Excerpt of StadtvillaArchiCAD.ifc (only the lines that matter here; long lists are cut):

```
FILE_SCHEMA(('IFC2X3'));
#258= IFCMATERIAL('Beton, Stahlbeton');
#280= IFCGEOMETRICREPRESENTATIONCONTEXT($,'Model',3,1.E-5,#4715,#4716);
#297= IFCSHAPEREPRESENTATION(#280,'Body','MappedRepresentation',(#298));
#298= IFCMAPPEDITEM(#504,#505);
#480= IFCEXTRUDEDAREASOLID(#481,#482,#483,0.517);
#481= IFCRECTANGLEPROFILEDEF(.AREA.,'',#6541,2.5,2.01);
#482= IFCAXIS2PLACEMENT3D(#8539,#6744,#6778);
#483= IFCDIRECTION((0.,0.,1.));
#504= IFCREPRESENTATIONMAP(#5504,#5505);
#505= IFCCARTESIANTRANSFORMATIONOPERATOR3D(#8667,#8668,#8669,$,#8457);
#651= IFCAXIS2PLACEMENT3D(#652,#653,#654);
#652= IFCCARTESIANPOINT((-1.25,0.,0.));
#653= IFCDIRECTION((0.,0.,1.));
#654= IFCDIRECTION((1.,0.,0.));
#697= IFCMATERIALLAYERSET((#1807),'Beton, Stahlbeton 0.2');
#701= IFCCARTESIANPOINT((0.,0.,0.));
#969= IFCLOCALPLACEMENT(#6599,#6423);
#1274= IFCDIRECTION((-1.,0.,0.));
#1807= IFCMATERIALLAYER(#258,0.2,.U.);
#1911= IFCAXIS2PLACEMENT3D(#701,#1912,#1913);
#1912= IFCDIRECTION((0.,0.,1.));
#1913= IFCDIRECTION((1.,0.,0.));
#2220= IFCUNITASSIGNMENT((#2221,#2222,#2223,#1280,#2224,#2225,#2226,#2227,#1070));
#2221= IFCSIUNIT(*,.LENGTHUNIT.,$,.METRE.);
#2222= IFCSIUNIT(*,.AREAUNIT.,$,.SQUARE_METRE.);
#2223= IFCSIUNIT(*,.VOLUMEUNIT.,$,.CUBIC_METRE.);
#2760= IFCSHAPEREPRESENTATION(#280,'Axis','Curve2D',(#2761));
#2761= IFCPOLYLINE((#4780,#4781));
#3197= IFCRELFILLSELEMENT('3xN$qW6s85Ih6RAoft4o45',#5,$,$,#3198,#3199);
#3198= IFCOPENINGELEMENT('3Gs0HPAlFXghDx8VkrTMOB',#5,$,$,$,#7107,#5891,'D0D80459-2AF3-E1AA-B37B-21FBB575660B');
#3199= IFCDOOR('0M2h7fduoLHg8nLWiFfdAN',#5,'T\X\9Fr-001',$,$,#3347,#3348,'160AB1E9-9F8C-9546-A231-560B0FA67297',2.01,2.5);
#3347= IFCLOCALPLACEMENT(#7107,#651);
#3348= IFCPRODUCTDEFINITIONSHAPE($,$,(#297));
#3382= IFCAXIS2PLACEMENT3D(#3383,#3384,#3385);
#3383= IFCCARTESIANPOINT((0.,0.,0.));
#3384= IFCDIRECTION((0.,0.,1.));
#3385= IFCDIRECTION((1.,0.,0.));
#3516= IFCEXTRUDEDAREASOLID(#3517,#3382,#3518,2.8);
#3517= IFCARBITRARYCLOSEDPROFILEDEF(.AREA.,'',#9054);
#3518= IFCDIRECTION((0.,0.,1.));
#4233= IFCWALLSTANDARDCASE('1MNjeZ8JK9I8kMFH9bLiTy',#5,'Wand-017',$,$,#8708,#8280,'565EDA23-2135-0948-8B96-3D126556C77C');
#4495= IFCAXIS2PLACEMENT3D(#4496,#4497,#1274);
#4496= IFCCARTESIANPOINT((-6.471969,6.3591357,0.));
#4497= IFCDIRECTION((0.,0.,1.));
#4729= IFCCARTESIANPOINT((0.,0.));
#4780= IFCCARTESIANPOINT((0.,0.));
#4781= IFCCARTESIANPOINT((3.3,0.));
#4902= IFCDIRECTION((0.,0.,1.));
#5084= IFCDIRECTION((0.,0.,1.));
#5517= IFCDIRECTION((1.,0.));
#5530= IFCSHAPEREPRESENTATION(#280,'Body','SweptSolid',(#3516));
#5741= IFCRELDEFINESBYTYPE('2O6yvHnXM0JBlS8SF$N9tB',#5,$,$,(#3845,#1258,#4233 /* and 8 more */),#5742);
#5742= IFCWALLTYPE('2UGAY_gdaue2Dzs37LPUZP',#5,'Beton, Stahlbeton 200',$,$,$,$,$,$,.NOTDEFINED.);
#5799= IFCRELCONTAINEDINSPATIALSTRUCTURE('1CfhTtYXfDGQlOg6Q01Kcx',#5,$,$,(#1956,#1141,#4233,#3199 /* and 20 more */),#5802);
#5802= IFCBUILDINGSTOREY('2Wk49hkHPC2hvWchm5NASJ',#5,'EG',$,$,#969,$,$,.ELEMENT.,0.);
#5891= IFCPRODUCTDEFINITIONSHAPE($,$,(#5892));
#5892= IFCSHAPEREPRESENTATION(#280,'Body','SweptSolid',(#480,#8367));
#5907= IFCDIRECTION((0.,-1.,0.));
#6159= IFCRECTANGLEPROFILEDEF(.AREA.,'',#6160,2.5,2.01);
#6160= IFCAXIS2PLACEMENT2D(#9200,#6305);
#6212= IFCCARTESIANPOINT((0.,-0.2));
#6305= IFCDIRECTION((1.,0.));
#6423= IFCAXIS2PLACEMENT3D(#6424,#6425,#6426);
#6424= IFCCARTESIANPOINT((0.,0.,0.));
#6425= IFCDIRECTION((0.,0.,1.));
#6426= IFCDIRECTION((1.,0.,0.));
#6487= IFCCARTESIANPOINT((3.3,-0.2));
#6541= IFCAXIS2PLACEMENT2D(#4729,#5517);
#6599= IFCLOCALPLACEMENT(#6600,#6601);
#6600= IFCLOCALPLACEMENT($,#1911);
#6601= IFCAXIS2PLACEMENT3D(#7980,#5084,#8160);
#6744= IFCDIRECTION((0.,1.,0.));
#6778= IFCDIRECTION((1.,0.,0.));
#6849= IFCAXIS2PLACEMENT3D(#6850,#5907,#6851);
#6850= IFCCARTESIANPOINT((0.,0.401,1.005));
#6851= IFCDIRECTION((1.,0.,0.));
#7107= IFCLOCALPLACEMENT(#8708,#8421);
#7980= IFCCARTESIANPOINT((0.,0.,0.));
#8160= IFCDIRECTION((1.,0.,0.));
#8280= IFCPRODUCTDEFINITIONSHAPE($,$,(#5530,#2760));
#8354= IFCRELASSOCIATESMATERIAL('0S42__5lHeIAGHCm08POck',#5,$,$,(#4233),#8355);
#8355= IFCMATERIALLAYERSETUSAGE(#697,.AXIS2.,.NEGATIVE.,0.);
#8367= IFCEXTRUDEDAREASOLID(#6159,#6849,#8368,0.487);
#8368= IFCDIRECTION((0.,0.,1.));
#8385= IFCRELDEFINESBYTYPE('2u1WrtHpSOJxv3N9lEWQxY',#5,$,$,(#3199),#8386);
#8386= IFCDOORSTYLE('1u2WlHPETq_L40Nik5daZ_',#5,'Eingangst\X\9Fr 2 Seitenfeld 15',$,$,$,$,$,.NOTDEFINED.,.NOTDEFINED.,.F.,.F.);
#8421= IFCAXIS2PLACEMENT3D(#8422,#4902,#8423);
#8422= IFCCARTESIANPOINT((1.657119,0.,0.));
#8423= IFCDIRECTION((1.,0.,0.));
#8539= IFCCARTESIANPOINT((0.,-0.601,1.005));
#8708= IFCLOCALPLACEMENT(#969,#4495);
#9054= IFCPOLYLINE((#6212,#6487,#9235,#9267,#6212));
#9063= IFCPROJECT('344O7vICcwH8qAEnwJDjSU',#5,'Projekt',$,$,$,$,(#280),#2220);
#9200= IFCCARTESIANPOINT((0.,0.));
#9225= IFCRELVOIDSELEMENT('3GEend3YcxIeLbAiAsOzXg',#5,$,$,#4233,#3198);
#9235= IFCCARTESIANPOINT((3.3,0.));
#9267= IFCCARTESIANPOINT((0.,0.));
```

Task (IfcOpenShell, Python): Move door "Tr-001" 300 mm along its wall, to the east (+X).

```python
import ifcopenshell
import ifcopenshell.api.geometry
import ifcopenshell.util.placement

model = ifcopenshell.open("StadtvillaArchiCAD.ifc")

door = model.by_id(3199)
opening = door.FillsVoids[0].RelatingOpeningElement
wall = opening.VoidsElements[0].RelatingBuildingElement

wall_matrix = ifcopenshell.util.placement.get_local_placement(wall.ObjectPlacement)
shift = wall_matrix[:3, 0] * -0.3
before = ifcopenshell.util.placement.get_local_placement(door.ObjectPlacement)[:3, 3].copy()

# The door is placed relative to its opening, so it follows when the opening moves.
matrix = ifcopenshell.util.placement.get_local_placement(opening.ObjectPlacement)
matrix[:3, 3] += shift
ifcopenshell.api.geometry.edit_object_placement(
    model, product=opening, matrix=matrix, is_si=False, should_transform_children=True
)

after = ifcopenshell.util.placement.get_local_placement(door.ObjectPlacement)[:3, 3]
print("door moved by", (after - before).round(3) + 0.0)

model.write("StadtvillaArchiCAD_edited.ifc")
```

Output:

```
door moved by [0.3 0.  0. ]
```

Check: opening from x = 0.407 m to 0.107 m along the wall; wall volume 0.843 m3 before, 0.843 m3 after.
